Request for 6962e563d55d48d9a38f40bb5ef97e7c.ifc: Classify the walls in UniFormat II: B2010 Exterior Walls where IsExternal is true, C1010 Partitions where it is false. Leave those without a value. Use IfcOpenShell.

First a look at what the model holds.

```python
import ifcopenshell
import ifcopenshell.util.element

model = ifcopenshell.open("6962e563d55d48d9a38f40bb5ef97e7c.ifc")
print(model.schema)
print("classifications:", [c.Name for c in model.by_type("IfcClassification")])
values = [ifcopenshell.util.element.get_pset(e, "Pset_WallCommon", "IsExternal") for e in model.by_type("IfcWall")]
for value in (True, False, None):
    print("IsExternal", value, values.count(value))
```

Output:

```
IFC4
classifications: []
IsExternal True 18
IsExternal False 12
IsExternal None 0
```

```python
import ifcopenshell
import ifcopenshell.api.classification
import ifcopenshell.util.element

model = ifcopenshell.open("6962e563d55d48d9a38f40bb5ef97e7c.ifc")

system = ifcopenshell.api.classification.add_classification(model, classification="UniFormat II")

walls = model.by_type("IfcWall")
external = {e: ifcopenshell.util.element.get_pset(e, "Pset_WallCommon", "IsExternal") for e in walls}
for flag, code, name in ((True, "B2010", "Exterior Walls"), (False, "C1010", "Partitions")):
    products = [e for e in walls if external[e] is flag]
    ifcopenshell.api.classification.add_reference(
        model, products=products, classification=system, identification=code, name=name
    )
    print(code, len(products))

model.write("6962e563d55d48d9a38f40bb5ef97e7c_edited.ifc")
```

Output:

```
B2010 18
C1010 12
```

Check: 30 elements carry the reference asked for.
